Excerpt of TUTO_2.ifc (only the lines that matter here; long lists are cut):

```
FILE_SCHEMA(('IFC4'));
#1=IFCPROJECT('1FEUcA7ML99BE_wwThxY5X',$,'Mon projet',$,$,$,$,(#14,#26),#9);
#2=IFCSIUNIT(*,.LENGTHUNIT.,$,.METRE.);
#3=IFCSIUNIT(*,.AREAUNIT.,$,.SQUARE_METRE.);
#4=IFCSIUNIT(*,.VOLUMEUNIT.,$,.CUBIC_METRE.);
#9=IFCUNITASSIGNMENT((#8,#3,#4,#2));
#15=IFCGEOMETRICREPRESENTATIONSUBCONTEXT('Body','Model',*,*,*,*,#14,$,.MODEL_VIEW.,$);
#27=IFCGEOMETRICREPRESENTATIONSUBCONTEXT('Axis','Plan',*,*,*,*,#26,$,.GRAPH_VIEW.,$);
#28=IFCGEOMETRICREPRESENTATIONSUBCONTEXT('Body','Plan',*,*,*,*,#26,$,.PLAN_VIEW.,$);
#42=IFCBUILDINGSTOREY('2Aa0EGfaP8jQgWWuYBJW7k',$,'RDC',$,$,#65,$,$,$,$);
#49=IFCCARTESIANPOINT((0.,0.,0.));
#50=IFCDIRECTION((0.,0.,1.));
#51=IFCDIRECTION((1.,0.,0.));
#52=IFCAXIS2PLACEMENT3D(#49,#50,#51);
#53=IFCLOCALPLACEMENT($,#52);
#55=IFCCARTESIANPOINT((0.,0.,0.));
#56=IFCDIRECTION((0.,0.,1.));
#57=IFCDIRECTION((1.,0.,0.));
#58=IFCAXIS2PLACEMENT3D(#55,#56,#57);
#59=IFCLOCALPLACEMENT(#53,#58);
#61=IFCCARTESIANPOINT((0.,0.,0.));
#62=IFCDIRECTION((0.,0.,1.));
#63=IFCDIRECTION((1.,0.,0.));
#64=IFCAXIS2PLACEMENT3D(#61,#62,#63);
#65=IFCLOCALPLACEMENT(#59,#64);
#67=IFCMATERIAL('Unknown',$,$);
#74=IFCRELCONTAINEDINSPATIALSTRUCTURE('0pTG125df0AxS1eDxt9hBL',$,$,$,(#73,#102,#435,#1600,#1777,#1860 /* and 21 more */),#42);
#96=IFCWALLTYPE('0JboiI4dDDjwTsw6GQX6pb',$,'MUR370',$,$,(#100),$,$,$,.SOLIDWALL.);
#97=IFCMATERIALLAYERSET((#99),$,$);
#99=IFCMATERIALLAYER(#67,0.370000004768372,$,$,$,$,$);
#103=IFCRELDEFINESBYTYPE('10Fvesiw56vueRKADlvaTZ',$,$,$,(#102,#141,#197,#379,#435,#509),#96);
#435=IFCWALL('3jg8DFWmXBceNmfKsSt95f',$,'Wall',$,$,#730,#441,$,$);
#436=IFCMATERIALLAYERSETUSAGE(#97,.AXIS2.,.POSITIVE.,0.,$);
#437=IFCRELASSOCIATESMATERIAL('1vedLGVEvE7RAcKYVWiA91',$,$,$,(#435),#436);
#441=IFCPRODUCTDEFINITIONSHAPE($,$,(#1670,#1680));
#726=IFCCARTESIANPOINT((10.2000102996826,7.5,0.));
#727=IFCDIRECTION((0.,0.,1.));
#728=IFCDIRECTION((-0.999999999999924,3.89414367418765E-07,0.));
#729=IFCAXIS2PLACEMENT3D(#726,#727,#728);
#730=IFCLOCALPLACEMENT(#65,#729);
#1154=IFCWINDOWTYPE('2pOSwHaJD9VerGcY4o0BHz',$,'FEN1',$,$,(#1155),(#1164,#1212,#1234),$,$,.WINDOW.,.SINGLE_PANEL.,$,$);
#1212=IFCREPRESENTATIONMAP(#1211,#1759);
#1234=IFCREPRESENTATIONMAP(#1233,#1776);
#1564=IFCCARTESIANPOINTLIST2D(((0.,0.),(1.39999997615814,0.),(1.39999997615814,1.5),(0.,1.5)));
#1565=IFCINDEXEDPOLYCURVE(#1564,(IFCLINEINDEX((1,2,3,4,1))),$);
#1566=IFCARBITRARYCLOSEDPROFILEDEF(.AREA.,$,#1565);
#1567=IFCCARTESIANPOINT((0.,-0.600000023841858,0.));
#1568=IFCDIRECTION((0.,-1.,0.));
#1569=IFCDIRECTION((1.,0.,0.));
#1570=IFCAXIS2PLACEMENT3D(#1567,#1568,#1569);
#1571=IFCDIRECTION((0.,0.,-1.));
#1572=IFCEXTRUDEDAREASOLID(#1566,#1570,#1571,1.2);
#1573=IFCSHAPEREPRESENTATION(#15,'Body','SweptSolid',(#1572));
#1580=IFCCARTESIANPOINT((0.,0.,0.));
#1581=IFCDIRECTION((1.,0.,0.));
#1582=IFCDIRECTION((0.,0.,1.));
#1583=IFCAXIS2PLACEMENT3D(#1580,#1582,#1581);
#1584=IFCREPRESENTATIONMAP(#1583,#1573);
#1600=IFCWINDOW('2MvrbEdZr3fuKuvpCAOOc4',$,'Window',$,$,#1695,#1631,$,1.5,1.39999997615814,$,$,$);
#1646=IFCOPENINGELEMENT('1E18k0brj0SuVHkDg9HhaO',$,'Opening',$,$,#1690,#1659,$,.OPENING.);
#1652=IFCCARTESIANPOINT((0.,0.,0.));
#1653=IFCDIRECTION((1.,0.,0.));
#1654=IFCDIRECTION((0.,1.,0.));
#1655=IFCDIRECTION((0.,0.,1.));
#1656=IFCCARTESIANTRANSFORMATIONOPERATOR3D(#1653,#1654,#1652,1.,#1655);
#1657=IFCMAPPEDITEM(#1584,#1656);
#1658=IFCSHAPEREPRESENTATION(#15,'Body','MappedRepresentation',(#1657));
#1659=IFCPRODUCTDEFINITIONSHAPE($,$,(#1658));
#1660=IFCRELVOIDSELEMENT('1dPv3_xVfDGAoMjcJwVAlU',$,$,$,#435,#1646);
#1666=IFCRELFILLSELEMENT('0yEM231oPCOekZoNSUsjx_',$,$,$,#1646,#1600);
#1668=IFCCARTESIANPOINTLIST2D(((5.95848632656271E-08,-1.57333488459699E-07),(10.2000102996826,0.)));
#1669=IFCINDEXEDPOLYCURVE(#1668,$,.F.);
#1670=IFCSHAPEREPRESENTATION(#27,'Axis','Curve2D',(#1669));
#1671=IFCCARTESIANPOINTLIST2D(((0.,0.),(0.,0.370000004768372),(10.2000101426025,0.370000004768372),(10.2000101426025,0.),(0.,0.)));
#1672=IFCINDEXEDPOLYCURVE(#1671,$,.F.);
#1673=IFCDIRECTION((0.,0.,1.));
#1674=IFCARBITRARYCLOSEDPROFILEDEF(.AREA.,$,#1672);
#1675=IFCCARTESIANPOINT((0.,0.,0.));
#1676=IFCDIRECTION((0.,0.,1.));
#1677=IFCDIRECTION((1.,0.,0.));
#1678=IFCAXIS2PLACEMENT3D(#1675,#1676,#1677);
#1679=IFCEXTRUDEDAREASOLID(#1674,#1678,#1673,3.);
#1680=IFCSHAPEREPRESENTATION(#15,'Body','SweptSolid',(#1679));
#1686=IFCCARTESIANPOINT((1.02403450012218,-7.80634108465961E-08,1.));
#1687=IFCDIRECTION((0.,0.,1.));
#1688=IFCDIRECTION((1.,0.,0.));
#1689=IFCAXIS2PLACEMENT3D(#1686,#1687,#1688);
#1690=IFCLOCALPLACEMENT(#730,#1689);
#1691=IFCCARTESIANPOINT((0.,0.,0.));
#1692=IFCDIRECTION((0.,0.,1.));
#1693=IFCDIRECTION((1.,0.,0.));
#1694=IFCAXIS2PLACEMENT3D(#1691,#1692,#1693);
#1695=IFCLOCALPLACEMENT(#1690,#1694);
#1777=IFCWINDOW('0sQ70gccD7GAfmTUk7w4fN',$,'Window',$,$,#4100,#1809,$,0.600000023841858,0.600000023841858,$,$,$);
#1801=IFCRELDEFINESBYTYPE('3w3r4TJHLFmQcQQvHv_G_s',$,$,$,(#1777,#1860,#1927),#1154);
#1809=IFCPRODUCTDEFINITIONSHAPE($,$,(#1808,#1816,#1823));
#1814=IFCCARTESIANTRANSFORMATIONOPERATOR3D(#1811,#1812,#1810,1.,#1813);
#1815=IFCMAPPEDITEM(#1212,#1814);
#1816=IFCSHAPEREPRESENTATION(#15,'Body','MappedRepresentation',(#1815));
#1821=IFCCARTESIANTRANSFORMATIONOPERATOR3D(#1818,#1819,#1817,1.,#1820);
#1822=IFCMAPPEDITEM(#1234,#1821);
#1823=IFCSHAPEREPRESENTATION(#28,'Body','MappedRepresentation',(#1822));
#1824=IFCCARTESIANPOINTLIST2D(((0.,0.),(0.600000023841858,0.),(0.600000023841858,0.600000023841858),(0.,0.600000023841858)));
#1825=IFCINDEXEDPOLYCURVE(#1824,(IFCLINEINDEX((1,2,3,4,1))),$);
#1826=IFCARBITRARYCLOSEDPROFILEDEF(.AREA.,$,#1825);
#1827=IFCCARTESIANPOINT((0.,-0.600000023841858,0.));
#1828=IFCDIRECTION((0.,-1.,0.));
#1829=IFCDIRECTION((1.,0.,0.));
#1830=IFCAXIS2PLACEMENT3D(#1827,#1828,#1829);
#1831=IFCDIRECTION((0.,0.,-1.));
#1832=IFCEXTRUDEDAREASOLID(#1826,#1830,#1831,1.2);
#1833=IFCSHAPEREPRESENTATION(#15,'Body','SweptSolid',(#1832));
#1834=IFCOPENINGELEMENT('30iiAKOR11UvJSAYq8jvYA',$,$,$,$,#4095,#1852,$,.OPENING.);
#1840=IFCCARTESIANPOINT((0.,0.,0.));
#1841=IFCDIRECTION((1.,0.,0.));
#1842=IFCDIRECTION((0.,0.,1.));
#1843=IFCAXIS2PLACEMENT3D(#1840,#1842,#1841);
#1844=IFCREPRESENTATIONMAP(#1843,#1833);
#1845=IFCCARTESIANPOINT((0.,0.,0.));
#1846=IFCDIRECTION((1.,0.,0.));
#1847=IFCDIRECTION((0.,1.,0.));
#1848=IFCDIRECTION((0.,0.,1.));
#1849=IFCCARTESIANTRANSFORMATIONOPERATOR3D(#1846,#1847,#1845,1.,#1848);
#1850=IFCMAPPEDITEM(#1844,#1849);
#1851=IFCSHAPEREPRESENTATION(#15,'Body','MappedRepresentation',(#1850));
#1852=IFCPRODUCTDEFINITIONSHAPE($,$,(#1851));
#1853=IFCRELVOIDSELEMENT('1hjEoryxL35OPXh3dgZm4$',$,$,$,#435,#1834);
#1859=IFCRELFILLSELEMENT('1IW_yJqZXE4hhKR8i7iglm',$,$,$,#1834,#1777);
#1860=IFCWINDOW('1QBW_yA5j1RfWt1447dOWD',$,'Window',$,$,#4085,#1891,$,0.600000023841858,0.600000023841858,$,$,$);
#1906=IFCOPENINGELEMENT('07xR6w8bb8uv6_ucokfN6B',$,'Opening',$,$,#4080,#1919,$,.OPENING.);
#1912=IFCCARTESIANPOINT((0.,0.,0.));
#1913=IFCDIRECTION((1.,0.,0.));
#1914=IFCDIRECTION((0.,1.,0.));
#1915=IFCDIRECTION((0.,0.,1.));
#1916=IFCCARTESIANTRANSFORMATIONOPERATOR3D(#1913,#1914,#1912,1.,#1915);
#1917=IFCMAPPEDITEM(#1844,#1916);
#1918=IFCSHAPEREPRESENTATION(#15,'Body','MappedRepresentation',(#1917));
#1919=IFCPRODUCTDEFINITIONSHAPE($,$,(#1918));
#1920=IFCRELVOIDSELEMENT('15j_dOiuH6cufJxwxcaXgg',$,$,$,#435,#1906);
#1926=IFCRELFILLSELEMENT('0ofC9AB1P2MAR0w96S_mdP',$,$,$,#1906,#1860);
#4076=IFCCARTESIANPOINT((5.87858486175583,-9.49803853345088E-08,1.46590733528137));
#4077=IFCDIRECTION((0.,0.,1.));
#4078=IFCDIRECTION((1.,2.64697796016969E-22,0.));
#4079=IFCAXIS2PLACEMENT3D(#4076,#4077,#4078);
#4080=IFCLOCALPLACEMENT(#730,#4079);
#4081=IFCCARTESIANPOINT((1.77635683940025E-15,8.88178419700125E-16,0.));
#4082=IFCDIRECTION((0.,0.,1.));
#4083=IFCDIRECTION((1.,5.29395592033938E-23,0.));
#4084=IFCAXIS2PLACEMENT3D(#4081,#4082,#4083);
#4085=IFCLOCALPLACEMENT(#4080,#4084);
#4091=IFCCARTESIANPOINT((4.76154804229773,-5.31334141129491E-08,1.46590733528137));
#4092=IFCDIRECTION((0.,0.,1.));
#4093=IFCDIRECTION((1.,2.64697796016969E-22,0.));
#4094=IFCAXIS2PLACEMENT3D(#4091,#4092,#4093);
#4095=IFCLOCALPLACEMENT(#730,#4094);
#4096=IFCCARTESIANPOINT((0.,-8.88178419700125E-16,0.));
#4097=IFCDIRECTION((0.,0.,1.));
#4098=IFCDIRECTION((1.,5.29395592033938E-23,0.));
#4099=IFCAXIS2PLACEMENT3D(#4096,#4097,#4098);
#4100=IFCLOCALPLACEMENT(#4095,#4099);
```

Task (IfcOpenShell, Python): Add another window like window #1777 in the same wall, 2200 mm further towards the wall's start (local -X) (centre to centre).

```python
import ifcopenshell
import ifcopenshell.api.feature
import ifcopenshell.api.geometry
import ifcopenshell.api.root
import ifcopenshell.geom
import ifcopenshell.util.element
import ifcopenshell.util.placement
import ifcopenshell.util.shape
import ifcopenshell.util.unit

model = ifcopenshell.open("TUTO_2.ifc")
unit_scale = ifcopenshell.util.unit.calculate_unit_scale(model)
settings = ifcopenshell.geom.settings()


def volume(element):
    """Net volume in cubic metres, openings subtracted."""
    shape = ifcopenshell.geom.create_shape(settings, element)
    return ifcopenshell.util.shape.get_volume(shape.geometry)


window = model.by_id(1777)
opening = window.FillsVoids[0].RelatingOpeningElement
wall = opening.VoidsElements[0].RelatingBuildingElement
before = volume(wall)
shift = ifcopenshell.util.placement.get_local_placement(wall.ObjectPlacement)[:3, 0] * -2.2 / unit_scale

# copy_class copies the void relationship, type, container and properties, but no geometry.
new_opening = ifcopenshell.api.root.copy_class(model, product=opening)
new_opening.Representation = ifcopenshell.util.element.copy_deep(
    model, opening.Representation, exclude=["IfcGeometricRepresentationContext", "IfcRepresentationMap"]
)
new_window = ifcopenshell.api.root.copy_class(model, product=window)
new_window.Representation = ifcopenshell.util.element.copy_deep(
    model, window.Representation, exclude=["IfcGeometricRepresentationContext", "IfcRepresentationMap"]
)
ifcopenshell.api.feature.add_filling(model, opening=new_opening, element=new_window)

for old, new in ((opening, new_opening), (window, new_window)):
    matrix = ifcopenshell.util.placement.get_local_placement(old.ObjectPlacement)
    matrix[:3, 3] += shift
    ifcopenshell.api.geometry.edit_object_placement(model, product=new, matrix=matrix, is_si=False)

after = volume(wall)

print(f"wall volume {before:.3f} -> {after:.3f} m3")

model.write("TUTO_2-out.ifc")
```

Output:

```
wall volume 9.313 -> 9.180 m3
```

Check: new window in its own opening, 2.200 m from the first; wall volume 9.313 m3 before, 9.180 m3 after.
